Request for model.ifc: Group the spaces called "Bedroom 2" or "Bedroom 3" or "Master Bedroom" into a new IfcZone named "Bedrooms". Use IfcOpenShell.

First a look at what the model holds.

```python
import ifcopenshell

model = ifcopenshell.open("model.ifc")
print(model.schema)
seen = {}
for space in model.by_type("IfcSpace"):
    seen[space.LongName] = seen.get(space.LongName, 0) + 1
for name, count in sorted(seen.items(), key=str):
    print(count, "x", name)
print("zones:", [z.Name for z in model.by_type("IfcZone")][:20])
```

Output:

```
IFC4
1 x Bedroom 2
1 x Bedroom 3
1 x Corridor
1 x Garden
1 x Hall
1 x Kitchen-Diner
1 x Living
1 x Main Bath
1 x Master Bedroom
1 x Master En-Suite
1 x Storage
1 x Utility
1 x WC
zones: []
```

```python
import ifcopenshell
import ifcopenshell.api.group
import ifcopenshell.api.root

model = ifcopenshell.open("model.ifc")

names = {"Bedroom 2", "Bedroom 3", "Master Bedroom"}
spaces = [s for s in model.by_type("IfcSpace") if s.LongName in names]

zone = ifcopenshell.api.root.create_entity(model, ifc_class="IfcZone", name="Bedrooms")
ifcopenshell.api.group.assign_group(model, products=spaces, group=zone)
print(len(spaces), "spaces in", zone.Name)

model.write("model_updated.ifc")
```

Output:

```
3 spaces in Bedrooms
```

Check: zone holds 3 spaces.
